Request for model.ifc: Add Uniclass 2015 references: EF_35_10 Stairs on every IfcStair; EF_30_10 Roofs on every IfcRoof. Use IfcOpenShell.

First a look at what the model holds.

```python
import ifcopenshell

model = ifcopenshell.open("model.ifc")
print(model.schema)
print("classifications:", [c.Name for c in model.by_type("IfcClassification")])
for ifc_class in ("IfcDoor", "IfcRoof", "IfcStair", "IfcWall", "IfcWindow"):
    print(ifc_class, len(model.by_type(ifc_class)))
```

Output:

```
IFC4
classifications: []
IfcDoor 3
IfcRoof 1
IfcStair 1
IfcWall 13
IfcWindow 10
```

```python
import ifcopenshell
import ifcopenshell.api.classification

model = ifcopenshell.open("model.ifc")

system = ifcopenshell.api.classification.add_classification(model, classification="Uniclass 2015")

codes = {
    "IfcStair": ("EF_35_10", "Stairs"),
    "IfcRoof": ("EF_30_10", "Roofs"),
}
for ifc_class, (code, name) in codes.items():
    products = model.by_type(ifc_class)
    ifcopenshell.api.classification.add_reference(
        model, products=products, classification=system, identification=code, name=name
    )
    print(code, len(products))

model.write("model_rev.ifc")
```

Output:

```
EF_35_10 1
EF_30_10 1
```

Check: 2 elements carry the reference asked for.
